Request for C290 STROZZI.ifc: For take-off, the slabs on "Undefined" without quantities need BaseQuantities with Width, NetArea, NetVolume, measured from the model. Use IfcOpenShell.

First a look at what the model holds.

```python
import ifcopenshell
import ifcopenshell.util.element
import ifcopenshell.util.unit

model = ifcopenshell.open("C290 STROZZI.ifc")
print(model.schema)
for unit_type in ("LENGTHUNIT", "AREAUNIT", "VOLUMEUNIT"):
    print(unit_type, ifcopenshell.util.unit.calculate_unit_scale(model, unit_type))
storey = next(s for s in model.by_type("IfcBuildingStorey") if s.Name == "Undefined")
slabs = [e for e in ifcopenshell.util.element.get_decomposition(storey) if e.is_a("IfcSlab")]
for e in sorted(slabs, key=lambda e: e.id()):
    print(e.id(), e.is_a(), e.Name, list(ifcopenshell.util.element.get_psets(e, qtos_only=True)), sep=" | ")
```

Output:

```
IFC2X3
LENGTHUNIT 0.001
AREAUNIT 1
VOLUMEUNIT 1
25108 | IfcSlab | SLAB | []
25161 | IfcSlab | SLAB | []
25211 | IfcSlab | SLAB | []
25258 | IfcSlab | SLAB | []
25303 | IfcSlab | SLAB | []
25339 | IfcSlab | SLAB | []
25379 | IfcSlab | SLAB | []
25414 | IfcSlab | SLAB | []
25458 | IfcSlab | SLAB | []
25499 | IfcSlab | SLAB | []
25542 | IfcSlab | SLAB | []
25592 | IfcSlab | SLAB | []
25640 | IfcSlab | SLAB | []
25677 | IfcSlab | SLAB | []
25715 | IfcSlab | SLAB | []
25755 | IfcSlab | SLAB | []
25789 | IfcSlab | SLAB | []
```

```python
import ifcopenshell
import ifcopenshell.api.pset
import ifcopenshell.geom
import ifcopenshell.util.element
import ifcopenshell.util.shape
import ifcopenshell.util.unit

model = ifcopenshell.open("C290 STROZZI.ifc")
unit_scale = ifcopenshell.util.unit.calculate_unit_scale(model)
area_scale = ifcopenshell.util.unit.calculate_unit_scale(model, "AREAUNIT")
volume_scale = ifcopenshell.util.unit.calculate_unit_scale(model, "VOLUMEUNIT")
settings = ifcopenshell.geom.settings()

storey = next(s for s in model.by_type("IfcBuildingStorey") if s.Name == "Undefined")
slabs = [e for e in ifcopenshell.util.element.get_decomposition(storey) if e.is_a("IfcSlab")]

for e in sorted(slabs, key=lambda e: e.id()):
    if ifcopenshell.util.element.get_psets(e, qtos_only=True, should_inherit=False):
        continue
    # Geometry comes back in metres, in the element's own axes.
    shape = ifcopenshell.geom.create_shape(settings, e)
    values = {
        "Width": ifcopenshell.util.shape.get_z(shape.geometry) / unit_scale,
        "NetArea": ifcopenshell.util.shape.get_footprint_area(shape.geometry) / area_scale,
        "NetVolume": ifcopenshell.util.shape.get_volume(shape.geometry) / volume_scale,
    }
    qto = ifcopenshell.api.pset.add_qto(model, product=e, name="BaseQuantities")
    ifcopenshell.api.pset.edit_qto(model, qto=qto, properties=values)
    print(e.id(), {k: round(v, 3) for k, v in values.items()})

model.write("C290 STROZZI_rev.ifc")
```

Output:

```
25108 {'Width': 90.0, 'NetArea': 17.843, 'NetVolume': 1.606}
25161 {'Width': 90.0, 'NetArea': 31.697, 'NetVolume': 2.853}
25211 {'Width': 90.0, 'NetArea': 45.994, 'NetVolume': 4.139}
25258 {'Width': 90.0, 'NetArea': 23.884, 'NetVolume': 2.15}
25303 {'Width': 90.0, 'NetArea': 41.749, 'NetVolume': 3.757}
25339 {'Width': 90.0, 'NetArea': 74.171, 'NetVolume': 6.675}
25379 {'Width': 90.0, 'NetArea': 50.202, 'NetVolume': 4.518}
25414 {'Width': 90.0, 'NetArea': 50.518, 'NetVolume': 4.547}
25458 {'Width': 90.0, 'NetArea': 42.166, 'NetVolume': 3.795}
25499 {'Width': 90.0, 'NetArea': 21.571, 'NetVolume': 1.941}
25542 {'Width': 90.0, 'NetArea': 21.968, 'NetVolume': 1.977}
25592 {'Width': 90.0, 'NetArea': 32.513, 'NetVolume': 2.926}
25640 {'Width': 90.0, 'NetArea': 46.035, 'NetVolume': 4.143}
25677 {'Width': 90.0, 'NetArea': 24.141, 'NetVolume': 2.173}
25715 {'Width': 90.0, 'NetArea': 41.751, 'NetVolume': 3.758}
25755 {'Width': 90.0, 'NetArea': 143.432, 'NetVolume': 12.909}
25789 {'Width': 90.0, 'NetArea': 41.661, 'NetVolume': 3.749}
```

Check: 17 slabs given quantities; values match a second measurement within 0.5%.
